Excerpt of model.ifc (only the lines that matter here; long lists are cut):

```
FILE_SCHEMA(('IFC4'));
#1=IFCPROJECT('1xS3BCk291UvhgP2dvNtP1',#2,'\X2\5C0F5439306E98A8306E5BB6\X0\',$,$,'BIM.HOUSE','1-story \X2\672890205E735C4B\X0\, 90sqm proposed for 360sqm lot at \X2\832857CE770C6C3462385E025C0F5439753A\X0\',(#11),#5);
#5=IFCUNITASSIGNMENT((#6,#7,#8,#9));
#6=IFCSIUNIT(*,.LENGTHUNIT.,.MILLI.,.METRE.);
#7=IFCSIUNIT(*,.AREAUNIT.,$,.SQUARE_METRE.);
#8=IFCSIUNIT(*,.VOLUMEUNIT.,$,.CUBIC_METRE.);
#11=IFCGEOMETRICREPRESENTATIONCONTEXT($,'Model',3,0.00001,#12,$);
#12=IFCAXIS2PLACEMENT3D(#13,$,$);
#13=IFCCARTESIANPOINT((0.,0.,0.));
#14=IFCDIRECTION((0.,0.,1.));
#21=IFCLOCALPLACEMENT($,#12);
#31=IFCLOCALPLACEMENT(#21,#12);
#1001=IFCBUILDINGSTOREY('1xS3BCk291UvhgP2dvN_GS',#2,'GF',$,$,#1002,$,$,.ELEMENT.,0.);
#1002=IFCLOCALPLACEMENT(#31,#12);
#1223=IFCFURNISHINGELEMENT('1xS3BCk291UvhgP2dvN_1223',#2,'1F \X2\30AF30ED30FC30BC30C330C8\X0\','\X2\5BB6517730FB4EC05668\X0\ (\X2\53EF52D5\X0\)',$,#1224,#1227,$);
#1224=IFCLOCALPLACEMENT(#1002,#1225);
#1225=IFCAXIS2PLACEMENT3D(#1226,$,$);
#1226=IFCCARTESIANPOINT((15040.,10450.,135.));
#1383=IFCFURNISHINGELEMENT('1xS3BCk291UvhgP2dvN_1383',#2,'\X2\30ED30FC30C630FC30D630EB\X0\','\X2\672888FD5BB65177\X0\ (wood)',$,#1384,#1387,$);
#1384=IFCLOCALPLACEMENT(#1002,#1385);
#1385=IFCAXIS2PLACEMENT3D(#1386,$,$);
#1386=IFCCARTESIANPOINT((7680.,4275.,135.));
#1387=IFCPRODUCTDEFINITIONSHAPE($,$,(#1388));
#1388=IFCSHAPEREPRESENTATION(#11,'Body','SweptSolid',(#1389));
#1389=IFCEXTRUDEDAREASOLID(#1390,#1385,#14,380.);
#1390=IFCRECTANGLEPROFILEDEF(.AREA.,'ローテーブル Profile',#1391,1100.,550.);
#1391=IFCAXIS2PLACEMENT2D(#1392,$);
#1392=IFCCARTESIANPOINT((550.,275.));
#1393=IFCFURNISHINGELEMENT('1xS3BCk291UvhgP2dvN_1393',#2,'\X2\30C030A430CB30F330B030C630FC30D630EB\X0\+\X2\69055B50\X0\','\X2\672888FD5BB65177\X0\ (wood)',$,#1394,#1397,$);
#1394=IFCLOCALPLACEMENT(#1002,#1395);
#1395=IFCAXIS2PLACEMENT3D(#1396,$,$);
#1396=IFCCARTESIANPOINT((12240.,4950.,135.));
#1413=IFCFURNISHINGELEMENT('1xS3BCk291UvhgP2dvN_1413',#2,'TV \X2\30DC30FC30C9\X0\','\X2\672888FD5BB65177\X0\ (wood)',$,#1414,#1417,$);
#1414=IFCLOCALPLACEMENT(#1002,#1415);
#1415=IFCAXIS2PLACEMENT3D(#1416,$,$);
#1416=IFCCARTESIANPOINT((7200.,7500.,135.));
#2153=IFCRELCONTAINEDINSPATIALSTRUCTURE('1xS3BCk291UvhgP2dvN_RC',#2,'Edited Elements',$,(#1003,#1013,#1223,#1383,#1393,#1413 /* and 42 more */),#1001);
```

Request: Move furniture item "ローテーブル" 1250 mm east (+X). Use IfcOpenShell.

```python
import ifcopenshell
import ifcopenshell.api.geometry
import ifcopenshell.util.placement

model = ifcopenshell.open("model.ifc")

item = model.by_id(1383)
matrix = ifcopenshell.util.placement.get_local_placement(item.ObjectPlacement)
matrix[0, 3] += 1250.0
ifcopenshell.api.geometry.edit_object_placement(model, product=item, matrix=matrix, is_si=False)

print(ifcopenshell.util.placement.get_local_placement(item.ObjectPlacement).round(3) + 0.0)

model.write("model_rev.ifc")
```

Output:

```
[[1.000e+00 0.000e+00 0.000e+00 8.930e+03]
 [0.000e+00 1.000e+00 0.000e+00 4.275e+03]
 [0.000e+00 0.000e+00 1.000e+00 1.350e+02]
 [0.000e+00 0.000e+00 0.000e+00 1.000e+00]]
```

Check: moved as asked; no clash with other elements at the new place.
